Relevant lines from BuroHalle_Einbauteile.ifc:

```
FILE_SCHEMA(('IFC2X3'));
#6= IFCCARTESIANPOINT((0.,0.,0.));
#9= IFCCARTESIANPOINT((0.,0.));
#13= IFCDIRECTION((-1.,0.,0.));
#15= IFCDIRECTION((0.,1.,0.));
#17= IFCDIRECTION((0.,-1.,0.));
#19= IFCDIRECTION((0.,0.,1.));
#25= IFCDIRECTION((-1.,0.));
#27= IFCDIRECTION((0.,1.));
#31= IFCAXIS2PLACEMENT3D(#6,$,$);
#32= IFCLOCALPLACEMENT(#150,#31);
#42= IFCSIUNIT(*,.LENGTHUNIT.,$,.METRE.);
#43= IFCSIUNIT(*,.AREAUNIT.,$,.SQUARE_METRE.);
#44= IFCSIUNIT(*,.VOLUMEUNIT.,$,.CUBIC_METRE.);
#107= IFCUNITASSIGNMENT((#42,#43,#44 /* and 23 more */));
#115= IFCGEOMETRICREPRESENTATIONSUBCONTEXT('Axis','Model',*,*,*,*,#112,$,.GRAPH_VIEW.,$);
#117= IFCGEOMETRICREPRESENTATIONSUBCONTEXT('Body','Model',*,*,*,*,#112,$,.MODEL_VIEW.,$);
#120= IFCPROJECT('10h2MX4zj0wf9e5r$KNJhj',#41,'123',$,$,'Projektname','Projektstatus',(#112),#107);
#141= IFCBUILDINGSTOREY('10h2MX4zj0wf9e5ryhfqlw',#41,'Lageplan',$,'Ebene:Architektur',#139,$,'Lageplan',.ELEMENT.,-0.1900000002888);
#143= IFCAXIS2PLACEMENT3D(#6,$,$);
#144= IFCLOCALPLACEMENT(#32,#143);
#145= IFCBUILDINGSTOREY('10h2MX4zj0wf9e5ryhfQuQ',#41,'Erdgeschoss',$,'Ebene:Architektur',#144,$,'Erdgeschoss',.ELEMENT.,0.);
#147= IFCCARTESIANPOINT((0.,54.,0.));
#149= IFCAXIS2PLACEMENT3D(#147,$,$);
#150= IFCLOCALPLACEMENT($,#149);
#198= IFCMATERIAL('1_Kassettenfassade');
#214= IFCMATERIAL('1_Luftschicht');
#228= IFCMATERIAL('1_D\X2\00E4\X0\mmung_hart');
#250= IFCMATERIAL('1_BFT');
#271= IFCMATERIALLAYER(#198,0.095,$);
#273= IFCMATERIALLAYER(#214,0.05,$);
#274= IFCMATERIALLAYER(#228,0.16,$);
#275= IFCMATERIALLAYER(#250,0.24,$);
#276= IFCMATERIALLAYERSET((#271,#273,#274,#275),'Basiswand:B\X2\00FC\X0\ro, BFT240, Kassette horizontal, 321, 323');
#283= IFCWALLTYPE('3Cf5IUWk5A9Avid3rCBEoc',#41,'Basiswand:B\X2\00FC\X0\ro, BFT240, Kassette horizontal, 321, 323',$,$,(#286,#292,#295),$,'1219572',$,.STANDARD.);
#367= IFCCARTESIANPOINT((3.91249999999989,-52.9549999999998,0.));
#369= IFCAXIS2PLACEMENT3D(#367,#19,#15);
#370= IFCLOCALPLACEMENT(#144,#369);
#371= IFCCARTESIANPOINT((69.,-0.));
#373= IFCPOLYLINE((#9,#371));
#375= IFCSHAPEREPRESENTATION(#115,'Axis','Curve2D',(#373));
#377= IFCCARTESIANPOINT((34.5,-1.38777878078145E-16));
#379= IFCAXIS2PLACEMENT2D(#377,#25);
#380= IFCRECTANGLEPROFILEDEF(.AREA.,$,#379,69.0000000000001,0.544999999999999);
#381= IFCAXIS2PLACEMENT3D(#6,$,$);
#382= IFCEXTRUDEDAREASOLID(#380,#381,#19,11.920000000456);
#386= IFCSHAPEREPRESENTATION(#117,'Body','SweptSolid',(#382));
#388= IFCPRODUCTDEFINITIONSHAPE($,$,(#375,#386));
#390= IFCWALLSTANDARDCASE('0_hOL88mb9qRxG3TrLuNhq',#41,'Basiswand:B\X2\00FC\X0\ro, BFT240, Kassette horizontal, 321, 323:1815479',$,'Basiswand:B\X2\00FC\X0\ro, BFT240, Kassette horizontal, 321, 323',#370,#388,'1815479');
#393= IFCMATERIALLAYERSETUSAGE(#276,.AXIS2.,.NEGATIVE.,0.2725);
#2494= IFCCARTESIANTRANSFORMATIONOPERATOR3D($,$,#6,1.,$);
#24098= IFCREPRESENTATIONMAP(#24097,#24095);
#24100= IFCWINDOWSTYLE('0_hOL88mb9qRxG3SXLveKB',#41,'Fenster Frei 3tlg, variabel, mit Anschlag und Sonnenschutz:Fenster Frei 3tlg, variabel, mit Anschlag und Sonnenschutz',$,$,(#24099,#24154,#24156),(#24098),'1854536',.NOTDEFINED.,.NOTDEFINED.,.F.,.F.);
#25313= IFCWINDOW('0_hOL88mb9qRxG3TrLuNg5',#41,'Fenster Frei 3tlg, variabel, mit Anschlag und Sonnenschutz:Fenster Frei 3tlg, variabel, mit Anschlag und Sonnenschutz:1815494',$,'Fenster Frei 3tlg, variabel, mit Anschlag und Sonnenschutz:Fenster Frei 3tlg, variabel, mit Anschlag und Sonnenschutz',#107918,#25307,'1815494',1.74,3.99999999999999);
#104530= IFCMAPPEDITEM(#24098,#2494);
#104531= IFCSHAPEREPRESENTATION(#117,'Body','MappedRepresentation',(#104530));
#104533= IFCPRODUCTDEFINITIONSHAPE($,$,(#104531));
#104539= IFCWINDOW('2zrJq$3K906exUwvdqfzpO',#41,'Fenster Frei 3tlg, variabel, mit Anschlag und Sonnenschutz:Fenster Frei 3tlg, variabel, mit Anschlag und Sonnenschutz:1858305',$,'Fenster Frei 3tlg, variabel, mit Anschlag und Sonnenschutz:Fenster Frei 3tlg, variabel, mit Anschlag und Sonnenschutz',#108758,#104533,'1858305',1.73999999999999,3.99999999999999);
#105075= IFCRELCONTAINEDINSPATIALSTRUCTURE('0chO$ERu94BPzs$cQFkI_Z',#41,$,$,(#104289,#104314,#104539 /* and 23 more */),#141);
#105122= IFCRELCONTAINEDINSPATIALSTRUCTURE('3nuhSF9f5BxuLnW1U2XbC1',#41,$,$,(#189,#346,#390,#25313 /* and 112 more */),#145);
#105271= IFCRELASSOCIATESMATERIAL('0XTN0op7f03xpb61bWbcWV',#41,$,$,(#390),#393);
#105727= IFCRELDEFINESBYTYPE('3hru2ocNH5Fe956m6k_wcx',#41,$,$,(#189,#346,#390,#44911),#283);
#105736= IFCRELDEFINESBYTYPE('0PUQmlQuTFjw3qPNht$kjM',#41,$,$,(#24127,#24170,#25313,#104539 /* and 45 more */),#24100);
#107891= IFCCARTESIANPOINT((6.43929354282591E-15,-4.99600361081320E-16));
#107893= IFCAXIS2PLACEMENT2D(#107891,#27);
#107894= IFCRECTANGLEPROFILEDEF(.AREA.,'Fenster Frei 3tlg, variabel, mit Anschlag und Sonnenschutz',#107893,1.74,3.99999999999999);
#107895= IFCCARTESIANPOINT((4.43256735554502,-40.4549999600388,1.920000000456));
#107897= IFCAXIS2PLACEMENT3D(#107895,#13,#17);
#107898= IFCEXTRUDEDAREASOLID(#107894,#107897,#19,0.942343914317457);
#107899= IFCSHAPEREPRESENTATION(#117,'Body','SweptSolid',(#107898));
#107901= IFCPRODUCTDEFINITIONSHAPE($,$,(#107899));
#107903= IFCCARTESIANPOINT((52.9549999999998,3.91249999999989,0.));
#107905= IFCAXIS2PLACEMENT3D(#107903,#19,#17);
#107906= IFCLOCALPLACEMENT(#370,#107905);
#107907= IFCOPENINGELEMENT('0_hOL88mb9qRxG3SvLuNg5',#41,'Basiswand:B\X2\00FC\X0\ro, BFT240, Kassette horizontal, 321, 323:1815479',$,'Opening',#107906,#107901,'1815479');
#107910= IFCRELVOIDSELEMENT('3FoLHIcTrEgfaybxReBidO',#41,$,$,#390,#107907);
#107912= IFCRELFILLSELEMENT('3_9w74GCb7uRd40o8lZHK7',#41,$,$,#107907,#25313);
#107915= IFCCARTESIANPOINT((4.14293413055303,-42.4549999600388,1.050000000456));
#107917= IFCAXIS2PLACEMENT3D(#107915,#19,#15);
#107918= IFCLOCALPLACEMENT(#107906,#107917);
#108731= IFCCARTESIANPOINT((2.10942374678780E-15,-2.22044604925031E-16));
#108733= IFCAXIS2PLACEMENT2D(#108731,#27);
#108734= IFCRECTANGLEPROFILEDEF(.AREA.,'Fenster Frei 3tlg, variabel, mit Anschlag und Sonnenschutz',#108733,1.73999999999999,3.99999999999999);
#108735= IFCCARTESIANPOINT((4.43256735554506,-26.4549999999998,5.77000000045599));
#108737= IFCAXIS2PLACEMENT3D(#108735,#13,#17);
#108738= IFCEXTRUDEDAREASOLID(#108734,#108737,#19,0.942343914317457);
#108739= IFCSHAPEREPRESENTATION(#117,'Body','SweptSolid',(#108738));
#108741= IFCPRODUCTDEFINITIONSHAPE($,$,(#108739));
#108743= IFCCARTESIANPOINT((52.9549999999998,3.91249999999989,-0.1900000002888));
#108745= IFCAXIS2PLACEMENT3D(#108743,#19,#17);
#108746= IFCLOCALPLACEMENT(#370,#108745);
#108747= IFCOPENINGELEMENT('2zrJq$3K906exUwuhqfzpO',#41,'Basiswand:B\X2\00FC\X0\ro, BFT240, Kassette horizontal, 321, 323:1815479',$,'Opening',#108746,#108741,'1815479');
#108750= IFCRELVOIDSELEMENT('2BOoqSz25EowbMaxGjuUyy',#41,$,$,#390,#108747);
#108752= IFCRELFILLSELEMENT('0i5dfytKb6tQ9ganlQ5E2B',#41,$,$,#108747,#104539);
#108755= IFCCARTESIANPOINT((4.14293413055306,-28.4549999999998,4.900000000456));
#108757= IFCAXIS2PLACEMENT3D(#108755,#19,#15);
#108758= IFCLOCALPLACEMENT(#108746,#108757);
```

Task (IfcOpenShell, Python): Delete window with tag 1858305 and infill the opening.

```python
import ifcopenshell
import ifcopenshell.api.feature
import ifcopenshell.api.root
import ifcopenshell.geom
import ifcopenshell.util.shape

model = ifcopenshell.open("BuroHalle_Einbauteile.ifc")
settings = ifcopenshell.geom.settings()


def volume(element):
    """Net volume in cubic metres, openings subtracted."""
    shape = ifcopenshell.geom.create_shape(settings, element)
    return ifcopenshell.util.shape.get_volume(shape.geometry)


window = model.by_id(104539)
opening = window.FillsVoids[0].RelatingOpeningElement
wall = opening.VoidsElements[0].RelatingBuildingElement
before = volume(wall)

ifcopenshell.api.root.remove_product(model, product=window)
ifcopenshell.api.feature.remove_feature(model, feature=opening)

after = volume(wall)

print(f"wall volume {before:.3f} -> {after:.3f} m3")

model.write("BuroHalle_Einbauteile_edited.ifc")
```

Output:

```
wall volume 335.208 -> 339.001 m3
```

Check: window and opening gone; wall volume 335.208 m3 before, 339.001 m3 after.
